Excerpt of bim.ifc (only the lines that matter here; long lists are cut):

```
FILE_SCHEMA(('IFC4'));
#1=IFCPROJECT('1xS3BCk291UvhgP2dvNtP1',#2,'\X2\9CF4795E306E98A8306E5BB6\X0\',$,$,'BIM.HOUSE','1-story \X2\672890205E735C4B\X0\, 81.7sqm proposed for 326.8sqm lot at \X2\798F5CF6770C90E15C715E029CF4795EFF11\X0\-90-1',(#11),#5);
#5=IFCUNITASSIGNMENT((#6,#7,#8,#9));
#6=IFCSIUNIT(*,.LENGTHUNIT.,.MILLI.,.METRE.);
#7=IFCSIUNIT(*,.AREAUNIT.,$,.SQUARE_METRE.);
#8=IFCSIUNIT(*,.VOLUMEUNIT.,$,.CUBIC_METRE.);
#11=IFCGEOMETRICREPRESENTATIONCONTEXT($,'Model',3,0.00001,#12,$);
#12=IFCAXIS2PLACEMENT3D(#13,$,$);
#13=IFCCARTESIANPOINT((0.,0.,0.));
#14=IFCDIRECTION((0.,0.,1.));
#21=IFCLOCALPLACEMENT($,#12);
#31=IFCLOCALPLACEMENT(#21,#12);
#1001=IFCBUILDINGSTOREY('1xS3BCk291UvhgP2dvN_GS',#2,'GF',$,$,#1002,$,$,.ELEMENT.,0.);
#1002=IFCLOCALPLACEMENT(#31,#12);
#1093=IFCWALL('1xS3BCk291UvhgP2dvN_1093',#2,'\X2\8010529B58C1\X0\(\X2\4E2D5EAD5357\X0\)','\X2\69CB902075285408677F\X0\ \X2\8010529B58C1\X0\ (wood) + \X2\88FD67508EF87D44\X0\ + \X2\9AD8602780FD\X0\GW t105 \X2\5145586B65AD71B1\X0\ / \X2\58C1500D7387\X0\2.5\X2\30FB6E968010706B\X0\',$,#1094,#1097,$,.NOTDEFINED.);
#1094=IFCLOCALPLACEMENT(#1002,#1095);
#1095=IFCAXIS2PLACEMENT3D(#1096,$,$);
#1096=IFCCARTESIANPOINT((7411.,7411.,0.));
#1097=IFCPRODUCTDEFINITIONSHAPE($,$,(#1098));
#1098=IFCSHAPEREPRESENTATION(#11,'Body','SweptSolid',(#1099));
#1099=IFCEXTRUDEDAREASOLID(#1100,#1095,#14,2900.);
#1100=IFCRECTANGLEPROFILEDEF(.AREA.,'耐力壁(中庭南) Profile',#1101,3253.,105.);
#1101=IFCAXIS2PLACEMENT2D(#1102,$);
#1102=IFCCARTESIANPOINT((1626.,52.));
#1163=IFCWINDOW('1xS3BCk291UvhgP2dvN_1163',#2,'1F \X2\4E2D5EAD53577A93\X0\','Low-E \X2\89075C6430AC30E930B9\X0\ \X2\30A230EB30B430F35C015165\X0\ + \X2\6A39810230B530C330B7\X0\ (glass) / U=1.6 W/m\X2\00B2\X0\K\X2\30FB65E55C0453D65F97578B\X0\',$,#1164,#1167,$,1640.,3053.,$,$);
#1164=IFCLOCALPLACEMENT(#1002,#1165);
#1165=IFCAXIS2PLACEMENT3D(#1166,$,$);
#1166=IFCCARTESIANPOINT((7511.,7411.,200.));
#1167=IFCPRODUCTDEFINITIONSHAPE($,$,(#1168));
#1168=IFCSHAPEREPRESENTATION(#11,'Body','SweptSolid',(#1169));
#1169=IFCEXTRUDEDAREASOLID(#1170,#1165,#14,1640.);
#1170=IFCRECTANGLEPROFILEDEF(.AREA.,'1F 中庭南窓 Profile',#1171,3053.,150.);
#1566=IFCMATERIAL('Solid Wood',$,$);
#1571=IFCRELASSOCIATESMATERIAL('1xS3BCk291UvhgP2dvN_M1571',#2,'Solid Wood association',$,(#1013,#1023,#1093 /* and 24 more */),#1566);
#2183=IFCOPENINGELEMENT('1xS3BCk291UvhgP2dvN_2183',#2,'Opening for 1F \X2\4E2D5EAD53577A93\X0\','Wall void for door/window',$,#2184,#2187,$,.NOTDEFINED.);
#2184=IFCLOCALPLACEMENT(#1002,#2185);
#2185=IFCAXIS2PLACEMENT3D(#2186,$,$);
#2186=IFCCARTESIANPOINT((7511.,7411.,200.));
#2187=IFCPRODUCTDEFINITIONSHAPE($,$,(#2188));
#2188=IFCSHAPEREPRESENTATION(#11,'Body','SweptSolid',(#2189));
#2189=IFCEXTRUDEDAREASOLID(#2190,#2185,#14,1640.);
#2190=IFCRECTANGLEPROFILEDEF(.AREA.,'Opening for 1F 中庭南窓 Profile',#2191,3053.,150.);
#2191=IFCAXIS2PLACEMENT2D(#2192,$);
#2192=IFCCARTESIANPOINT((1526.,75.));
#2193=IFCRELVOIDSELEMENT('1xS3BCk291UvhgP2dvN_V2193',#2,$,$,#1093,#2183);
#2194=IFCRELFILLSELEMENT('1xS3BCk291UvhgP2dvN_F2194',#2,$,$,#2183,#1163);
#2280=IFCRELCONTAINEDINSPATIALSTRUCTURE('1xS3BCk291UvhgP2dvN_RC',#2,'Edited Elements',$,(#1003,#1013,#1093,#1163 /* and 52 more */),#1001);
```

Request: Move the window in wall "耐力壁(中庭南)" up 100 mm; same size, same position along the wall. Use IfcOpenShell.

```python
import numpy as np
import ifcopenshell
import ifcopenshell.api.geometry
import ifcopenshell.util.placement
import ifcopenshell.util.unit

model = ifcopenshell.open("bim.ifc")
unit_scale = ifcopenshell.util.unit.calculate_unit_scale(model)

window = model.by_guid("1xS3BCk291UvhgP2dvN_1163")
opening = window.FillsVoids[0].RelatingOpeningElement
dz = 0.1 / unit_scale

shift = np.array([0.0, 0.0, dz])
# The window is not placed relative to its opening, so move both.
for product in (opening, window):
    matrix = ifcopenshell.util.placement.get_local_placement(product.ObjectPlacement)
    matrix[:3, 3] += shift
    ifcopenshell.api.geometry.edit_object_placement(model, product=product, matrix=matrix, is_si=False)

print(f"moved by {dz * unit_scale:+.3f} m")

model.write("bim_edited.ifc")
```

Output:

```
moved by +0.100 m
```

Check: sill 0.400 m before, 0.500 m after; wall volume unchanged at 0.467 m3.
